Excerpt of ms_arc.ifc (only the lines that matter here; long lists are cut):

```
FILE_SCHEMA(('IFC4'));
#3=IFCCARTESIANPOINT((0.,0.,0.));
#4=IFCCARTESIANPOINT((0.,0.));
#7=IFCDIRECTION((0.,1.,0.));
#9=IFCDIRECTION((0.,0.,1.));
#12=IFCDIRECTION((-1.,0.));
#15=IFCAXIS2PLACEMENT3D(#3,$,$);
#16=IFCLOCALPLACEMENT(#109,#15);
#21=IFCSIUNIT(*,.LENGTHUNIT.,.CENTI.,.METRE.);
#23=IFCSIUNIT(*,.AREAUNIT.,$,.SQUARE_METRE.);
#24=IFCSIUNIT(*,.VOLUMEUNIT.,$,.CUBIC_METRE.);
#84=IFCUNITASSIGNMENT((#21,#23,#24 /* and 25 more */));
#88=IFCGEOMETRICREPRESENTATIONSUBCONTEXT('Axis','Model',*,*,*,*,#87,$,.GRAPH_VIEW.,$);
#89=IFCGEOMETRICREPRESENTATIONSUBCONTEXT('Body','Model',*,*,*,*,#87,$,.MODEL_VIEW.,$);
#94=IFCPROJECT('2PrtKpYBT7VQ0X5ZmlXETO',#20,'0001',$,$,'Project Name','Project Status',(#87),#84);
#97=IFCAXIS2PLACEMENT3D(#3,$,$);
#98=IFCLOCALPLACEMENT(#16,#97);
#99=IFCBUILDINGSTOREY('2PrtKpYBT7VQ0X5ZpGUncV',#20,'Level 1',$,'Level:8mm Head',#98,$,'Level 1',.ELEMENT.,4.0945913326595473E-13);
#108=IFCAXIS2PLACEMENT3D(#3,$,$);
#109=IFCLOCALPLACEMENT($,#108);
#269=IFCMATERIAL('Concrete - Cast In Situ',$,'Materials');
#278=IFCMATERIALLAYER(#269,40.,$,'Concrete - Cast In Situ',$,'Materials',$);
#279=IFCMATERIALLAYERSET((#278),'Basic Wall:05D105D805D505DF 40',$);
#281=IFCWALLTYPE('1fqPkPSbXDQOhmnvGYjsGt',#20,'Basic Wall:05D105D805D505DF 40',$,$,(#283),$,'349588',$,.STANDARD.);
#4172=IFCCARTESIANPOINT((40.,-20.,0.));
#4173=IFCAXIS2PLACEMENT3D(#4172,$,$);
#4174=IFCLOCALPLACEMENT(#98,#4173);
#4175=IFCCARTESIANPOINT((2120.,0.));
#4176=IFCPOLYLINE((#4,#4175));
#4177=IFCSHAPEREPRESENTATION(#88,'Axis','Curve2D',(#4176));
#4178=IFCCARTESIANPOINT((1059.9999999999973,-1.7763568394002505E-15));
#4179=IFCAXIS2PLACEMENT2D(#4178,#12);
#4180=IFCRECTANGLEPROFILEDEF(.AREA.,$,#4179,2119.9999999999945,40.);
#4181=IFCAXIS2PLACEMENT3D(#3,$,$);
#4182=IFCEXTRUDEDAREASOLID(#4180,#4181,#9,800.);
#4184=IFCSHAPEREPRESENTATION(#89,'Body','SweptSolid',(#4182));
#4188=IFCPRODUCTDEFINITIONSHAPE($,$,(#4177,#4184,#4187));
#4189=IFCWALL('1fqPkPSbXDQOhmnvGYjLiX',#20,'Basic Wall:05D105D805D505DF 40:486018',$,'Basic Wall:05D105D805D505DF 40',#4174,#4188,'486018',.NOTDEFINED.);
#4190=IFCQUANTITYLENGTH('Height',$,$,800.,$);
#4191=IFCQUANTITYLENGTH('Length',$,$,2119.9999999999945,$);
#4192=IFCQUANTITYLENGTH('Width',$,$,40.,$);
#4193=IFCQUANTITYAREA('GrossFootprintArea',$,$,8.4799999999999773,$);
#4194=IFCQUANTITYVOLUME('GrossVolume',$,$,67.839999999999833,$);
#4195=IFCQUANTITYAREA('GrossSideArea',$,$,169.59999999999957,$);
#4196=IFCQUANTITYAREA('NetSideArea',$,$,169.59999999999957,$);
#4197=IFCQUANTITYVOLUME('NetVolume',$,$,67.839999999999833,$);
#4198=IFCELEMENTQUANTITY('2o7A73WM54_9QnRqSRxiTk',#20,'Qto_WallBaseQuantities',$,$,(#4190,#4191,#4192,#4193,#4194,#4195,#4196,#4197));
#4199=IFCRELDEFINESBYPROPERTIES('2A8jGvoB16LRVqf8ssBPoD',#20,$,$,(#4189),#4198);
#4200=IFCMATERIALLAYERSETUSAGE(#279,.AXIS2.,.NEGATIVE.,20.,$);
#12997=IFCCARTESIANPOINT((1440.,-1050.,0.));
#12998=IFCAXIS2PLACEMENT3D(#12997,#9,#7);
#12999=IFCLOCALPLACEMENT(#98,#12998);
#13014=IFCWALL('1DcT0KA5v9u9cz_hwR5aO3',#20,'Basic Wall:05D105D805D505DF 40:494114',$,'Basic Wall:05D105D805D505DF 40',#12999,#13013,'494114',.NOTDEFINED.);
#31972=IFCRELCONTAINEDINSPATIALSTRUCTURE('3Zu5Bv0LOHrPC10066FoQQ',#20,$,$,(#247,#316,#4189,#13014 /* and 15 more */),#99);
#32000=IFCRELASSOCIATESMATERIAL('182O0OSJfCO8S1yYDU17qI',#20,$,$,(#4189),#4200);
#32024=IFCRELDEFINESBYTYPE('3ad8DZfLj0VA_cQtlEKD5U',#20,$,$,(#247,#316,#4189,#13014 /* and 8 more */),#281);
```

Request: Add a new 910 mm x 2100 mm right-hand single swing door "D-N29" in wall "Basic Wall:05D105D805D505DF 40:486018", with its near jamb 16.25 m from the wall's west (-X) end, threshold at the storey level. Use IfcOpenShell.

```python
import numpy as np
import ifcopenshell
import ifcopenshell.api.feature
import ifcopenshell.api.geometry
import ifcopenshell.api.pset
import ifcopenshell.api.root
import ifcopenshell.api.spatial
import ifcopenshell.geom
import ifcopenshell.util.element
import ifcopenshell.util.placement
import ifcopenshell.util.representation
import ifcopenshell.util.shape
import ifcopenshell.util.unit

model = ifcopenshell.open("ms_arc.ifc")
unit_scale = ifcopenshell.util.unit.calculate_unit_scale(model)
area_scale = ifcopenshell.util.unit.calculate_unit_scale(model, "AREAUNIT")
volume_scale = ifcopenshell.util.unit.calculate_unit_scale(model, "VOLUMEUNIT")
settings = ifcopenshell.geom.settings()


def volume(element):
    """Net volume in cubic metres, openings subtracted."""
    shape = ifcopenshell.geom.create_shape(settings, element)
    return ifcopenshell.util.shape.get_volume(shape.geometry)


wall = model.by_id(4189)
storey = ifcopenshell.util.element.get_container(wall, ifc_class="IfcBuildingStorey")
context = ifcopenshell.util.representation.get_context(model, "Model", "Body", "MODEL_VIEW")
before = volume(wall)

width, height, from_end, sill = 0.91, 2.1, 16.25, 0.0  # metres

# The wall runs along its own X axis, and the end named is its -X end.
wall_shape = ifcopenshell.geom.create_shape(settings, wall)
x, y, z = ifcopenshell.util.shape.get_vertices(wall_shape.geometry).T
start = x.min() + from_end
face, thickness = float(y.min()), float(y.max() - y.min())
wall_matrix = ifcopenshell.util.placement.get_local_placement(wall.ObjectPlacement)
level = ifcopenshell.util.placement.get_local_placement(storey.ObjectPlacement)[2, 3]


def in_wall(x, y):
    """Placement at x, y metres in the wall's axes, at sill height."""
    matrix = wall_matrix.copy()
    matrix[:, 3] = wall_matrix @ np.array([x / unit_scale, y / unit_scale, 0.0, 1.0])
    matrix[2, 3] = level + sill / unit_scale
    return matrix


# Opening: a box that overshoots both wall faces by 50 mm.
opening = ifcopenshell.api.root.create_entity(model, ifc_class="IfcOpeningElement", predefined_type="OPENING")
box = ifcopenshell.api.geometry.add_wall_representation(
    model, context=context, length=width, height=height, thickness=thickness + 0.1
)
ifcopenshell.api.geometry.assign_representation(model, product=opening, representation=box)
ifcopenshell.api.geometry.edit_object_placement(model, product=opening, matrix=in_wall(start, face - 0.05), is_si=False)
ifcopenshell.api.feature.add_feature(model, feature=opening, element=wall)

door = ifcopenshell.api.root.create_entity(model, ifc_class="IfcDoor", name="D-N29", predefined_type="DOOR")
door.OverallWidth, door.OverallHeight = width / unit_scale, height / unit_scale
door.OperationType = "SINGLE_SWING_RIGHT"
body = ifcopenshell.api.geometry.add_door_representation(
    model,
    context=context,
    overall_width=door.OverallWidth,
    overall_height=door.OverallHeight,
    operation_type="SINGLE_SWING_RIGHT",
    lining_properties={"LiningDepth": thickness / unit_scale, "ThresholdDepth": thickness / unit_scale},
)
ifcopenshell.api.geometry.assign_representation(model, product=door, representation=body)
ifcopenshell.api.spatial.assign_container(model, products=[door], relating_structure=storey)
ifcopenshell.api.feature.add_filling(model, opening=opening, element=door)

# The lining spans the wall, so the door starts at the wall face.
ifcopenshell.api.geometry.edit_object_placement(model, product=door, matrix=in_wall(start, face), is_si=False)

after = volume(wall)

# Update the wall's stored quantities.
qto = model.by_id(ifcopenshell.util.element.get_pset(wall, "Qto_WallBaseQuantities", should_inherit=False)["id"])
ifcopenshell.api.pset.edit_qto(model, qto=qto, properties={
    "NetSideArea": after / thickness / area_scale,
    "NetVolume": after / volume_scale,
})

print(f"wall volume {before:.3f} -> {after:.3f} m3")

model.write("ms_arc_edited.ifc")
```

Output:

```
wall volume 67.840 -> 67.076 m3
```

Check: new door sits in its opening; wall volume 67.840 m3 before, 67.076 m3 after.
